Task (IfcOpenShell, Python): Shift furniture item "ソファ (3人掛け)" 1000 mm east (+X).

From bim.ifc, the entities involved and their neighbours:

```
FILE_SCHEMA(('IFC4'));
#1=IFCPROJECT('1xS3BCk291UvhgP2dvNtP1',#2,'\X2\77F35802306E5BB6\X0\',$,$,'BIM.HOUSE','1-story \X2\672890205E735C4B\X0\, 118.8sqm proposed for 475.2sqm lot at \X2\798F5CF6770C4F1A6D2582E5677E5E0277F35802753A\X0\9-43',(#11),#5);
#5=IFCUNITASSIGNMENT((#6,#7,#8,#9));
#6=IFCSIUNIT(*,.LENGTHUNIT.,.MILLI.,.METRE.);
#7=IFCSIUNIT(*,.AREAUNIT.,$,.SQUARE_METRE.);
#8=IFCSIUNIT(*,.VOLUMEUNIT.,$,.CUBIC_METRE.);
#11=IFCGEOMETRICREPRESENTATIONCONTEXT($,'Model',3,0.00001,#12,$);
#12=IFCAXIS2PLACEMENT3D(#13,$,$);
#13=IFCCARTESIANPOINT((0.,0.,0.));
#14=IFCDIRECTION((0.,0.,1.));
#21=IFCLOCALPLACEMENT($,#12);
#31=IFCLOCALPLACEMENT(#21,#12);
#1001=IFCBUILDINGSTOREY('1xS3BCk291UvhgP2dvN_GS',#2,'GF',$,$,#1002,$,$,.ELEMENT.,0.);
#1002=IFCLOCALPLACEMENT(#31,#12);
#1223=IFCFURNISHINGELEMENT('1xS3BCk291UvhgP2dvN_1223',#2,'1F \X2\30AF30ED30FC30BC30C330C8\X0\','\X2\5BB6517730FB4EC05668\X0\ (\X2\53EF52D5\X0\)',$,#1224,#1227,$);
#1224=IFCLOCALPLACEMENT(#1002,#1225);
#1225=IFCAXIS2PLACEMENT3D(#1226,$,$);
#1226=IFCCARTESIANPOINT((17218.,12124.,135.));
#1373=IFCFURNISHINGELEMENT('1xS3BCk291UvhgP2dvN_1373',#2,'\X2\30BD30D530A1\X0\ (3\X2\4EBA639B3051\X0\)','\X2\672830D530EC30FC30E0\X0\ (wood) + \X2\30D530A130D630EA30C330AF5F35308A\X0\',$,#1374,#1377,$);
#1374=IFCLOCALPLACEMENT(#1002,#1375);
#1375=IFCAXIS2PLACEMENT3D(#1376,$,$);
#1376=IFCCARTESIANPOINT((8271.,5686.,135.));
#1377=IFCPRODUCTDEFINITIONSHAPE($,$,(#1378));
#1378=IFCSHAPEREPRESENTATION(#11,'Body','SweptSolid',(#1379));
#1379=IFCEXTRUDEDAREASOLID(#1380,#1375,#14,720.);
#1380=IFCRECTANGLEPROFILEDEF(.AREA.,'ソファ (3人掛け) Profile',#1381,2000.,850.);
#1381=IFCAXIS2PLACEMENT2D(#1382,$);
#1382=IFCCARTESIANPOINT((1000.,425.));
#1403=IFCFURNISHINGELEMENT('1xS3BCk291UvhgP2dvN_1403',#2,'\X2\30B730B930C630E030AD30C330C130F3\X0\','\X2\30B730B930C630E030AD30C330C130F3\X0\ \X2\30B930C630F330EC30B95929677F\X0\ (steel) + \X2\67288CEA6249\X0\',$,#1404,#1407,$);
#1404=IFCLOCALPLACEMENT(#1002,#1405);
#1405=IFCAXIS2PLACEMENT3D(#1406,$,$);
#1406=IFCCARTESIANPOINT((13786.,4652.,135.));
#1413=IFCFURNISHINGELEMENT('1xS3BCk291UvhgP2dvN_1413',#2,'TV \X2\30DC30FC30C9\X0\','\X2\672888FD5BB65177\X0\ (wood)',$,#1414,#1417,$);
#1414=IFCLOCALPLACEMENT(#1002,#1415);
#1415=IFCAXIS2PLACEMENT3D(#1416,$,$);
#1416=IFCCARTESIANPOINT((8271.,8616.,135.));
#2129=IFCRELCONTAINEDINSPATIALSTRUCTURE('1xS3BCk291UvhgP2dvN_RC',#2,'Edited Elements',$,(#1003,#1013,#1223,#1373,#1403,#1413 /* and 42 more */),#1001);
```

```python
import ifcopenshell
import ifcopenshell.api.geometry
import ifcopenshell.util.placement
import ifcopenshell.util.unit

model = ifcopenshell.open("bim.ifc")
unit_scale = ifcopenshell.util.unit.calculate_unit_scale(model)

item = model.by_guid("1xS3BCk291UvhgP2dvN_1373")
matrix = ifcopenshell.util.placement.get_local_placement(item.ObjectPlacement)
matrix[0, 3] += 1 / unit_scale
ifcopenshell.api.geometry.edit_object_placement(model, product=item, matrix=matrix, is_si=False)

print(ifcopenshell.util.placement.get_local_placement(item.ObjectPlacement).round(3) + 0.0)

model.write("bim_edited.ifc")
```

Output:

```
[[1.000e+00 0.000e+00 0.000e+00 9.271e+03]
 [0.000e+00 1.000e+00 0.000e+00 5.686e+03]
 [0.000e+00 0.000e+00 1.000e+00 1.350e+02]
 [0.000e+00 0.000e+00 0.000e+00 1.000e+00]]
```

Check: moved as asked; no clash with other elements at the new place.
